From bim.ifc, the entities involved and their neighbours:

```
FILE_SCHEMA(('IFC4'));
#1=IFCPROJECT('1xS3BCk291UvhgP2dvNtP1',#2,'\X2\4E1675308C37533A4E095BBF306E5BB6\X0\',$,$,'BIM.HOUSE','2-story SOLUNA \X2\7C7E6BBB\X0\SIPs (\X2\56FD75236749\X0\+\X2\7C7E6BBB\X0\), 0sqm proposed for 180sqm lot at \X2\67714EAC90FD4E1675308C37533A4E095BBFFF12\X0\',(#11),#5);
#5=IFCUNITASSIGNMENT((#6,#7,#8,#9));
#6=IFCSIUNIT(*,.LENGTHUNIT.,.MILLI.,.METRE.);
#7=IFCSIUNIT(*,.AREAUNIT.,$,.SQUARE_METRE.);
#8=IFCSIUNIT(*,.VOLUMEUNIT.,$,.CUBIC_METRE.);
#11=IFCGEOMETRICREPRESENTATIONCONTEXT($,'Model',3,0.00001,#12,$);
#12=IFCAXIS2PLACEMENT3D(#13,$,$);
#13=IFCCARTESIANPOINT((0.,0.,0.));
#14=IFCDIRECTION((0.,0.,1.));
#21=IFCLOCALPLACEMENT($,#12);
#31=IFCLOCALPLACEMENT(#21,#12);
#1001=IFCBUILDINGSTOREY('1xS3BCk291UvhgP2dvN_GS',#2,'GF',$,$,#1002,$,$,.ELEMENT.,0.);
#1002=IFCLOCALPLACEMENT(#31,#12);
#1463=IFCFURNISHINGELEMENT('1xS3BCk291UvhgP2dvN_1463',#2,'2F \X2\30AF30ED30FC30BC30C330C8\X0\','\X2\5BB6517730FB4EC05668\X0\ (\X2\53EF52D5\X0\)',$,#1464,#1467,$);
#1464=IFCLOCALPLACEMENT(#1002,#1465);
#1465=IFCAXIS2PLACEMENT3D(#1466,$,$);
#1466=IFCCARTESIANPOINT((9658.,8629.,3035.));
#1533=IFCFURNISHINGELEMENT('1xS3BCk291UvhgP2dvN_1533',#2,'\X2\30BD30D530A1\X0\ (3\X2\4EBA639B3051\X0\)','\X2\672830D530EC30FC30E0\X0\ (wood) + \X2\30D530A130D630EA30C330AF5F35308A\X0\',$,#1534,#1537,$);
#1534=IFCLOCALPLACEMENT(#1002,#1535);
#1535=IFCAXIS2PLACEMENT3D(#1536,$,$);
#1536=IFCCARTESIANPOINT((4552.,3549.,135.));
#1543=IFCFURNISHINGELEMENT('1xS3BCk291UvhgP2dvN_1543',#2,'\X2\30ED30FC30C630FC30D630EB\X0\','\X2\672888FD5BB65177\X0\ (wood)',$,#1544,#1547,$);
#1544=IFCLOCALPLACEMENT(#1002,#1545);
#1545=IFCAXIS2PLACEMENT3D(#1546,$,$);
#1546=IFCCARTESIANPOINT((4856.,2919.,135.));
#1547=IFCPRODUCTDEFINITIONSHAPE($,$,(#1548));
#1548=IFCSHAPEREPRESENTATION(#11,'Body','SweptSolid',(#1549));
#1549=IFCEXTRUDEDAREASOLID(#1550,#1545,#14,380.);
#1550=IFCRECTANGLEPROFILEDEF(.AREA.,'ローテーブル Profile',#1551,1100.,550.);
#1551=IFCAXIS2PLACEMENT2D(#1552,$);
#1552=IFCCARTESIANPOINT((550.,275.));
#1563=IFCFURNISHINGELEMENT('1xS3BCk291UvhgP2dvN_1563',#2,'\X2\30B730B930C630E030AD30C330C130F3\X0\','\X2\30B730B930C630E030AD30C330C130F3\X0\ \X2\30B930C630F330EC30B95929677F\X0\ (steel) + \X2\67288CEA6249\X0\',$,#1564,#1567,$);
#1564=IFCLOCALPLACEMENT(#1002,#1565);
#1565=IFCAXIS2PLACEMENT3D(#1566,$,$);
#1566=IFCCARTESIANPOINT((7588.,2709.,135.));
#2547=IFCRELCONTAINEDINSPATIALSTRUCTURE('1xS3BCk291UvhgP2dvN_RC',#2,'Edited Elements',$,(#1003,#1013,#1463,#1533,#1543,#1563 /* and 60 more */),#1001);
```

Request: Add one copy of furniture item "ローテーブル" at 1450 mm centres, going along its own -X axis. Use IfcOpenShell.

```python
import ifcopenshell
import ifcopenshell.api.geometry
import ifcopenshell.api.root
import ifcopenshell.util.element
import ifcopenshell.util.placement

model = ifcopenshell.open("bim.ifc")


def reuse_history(source, copy):
    """copy_class also copies each property set's owner history, people and application; keep the originals."""
    for rel in copy.IsDefinedBy:
        if rel.is_a("IfcRelDefinesByProperties") and (history := rel.RelatingPropertyDefinition.OwnerHistory):
            rel.RelatingPropertyDefinition.OwnerHistory = source.OwnerHistory
            ifcopenshell.util.element.remove_deep2(model, history)


source = model.by_id(1543)
base = ifcopenshell.util.placement.get_local_placement(source.ObjectPlacement)
step = -base[:3, 0] * 1450.0

for i in range(1, 2):
    copy = ifcopenshell.api.root.copy_class(model, product=source)
    copy.Representation = ifcopenshell.util.element.copy_deep(
        model, source.Representation, exclude=["IfcGeometricRepresentationContext", "IfcRepresentationMap"]
    )
    reuse_history(source, copy)
    matrix = base.copy()
    matrix[:3, 3] += i * step
    print("added at", matrix[:3, 3].round(3) + 0.0)
    ifcopenshell.api.geometry.edit_object_placement(model, product=copy, matrix=matrix, is_si=False)

model.write("bim_rev.ifc")
```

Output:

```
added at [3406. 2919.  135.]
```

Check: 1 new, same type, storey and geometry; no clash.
